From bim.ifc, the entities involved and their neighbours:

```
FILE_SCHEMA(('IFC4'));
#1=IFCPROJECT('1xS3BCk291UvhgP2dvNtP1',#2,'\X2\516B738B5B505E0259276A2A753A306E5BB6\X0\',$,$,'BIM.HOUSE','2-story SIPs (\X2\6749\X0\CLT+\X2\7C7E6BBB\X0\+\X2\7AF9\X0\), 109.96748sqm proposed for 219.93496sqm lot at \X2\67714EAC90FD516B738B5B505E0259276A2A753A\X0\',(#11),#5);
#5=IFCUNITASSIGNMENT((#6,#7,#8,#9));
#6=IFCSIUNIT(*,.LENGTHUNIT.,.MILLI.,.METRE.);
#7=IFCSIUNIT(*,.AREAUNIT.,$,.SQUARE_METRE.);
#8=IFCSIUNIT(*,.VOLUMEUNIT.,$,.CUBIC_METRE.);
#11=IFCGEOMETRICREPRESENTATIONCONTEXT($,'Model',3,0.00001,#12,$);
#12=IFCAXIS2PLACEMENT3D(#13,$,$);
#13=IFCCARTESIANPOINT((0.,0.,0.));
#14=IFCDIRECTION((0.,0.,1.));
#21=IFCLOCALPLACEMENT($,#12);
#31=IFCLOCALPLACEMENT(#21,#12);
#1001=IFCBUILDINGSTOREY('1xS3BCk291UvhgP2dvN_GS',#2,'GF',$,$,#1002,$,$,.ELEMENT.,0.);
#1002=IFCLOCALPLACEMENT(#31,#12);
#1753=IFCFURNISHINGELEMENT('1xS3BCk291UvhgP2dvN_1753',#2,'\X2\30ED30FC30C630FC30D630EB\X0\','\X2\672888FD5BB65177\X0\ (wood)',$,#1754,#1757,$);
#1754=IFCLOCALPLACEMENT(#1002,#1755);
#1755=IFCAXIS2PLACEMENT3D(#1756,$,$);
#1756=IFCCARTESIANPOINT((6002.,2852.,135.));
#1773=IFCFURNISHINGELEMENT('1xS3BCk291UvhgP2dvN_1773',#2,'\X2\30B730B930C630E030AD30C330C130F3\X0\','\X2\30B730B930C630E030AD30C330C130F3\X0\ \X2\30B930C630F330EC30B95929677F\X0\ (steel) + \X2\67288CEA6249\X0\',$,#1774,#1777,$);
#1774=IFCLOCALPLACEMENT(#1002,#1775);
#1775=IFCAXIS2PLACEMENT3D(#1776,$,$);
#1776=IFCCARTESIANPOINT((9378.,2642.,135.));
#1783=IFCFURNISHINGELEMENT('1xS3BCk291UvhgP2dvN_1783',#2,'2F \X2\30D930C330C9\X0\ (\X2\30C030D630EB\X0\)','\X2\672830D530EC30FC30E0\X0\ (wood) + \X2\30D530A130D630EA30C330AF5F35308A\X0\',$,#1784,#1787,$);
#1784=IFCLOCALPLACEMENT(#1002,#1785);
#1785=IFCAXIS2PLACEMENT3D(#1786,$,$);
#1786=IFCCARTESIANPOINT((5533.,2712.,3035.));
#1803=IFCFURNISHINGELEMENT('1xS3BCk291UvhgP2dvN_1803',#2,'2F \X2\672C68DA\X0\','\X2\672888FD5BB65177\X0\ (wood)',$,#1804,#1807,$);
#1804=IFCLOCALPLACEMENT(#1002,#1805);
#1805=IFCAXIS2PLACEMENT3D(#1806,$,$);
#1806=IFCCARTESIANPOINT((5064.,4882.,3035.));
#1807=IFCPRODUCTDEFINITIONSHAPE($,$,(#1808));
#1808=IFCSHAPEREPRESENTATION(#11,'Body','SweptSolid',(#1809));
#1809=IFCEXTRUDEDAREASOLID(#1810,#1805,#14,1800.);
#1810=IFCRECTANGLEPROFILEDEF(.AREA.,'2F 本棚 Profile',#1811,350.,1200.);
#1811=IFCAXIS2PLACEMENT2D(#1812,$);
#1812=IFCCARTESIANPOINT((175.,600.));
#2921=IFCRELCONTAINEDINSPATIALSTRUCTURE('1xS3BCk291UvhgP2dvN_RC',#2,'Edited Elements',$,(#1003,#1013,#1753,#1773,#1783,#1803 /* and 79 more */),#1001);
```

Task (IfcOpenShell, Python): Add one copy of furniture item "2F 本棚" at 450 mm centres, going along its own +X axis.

```python
import ifcopenshell
import ifcopenshell.api.geometry
import ifcopenshell.api.root
import ifcopenshell.util.element
import ifcopenshell.util.placement
import ifcopenshell.util.unit

model = ifcopenshell.open("bim.ifc")
unit_scale = ifcopenshell.util.unit.calculate_unit_scale(model)


def reuse_history(source, copy):
    """copy_class also copies each property set's owner history, people and application; keep the originals."""
    for rel in copy.IsDefinedBy:
        if rel.is_a("IfcRelDefinesByProperties") and (history := rel.RelatingPropertyDefinition.OwnerHistory):
            rel.RelatingPropertyDefinition.OwnerHistory = source.OwnerHistory
            ifcopenshell.util.element.remove_deep2(model, history)


source = model.by_id(1803)
base = ifcopenshell.util.placement.get_local_placement(source.ObjectPlacement)
step = base[:3, 0] * 0.45 / unit_scale

for i in range(1, 2):
    copy = ifcopenshell.api.root.copy_class(model, product=source)
    copy.Representation = ifcopenshell.util.element.copy_deep(
        model, source.Representation, exclude=["IfcGeometricRepresentationContext", "IfcRepresentationMap"]
    )
    reuse_history(source, copy)
    matrix = base.copy()
    matrix[:3, 3] += i * step
    print("added at", matrix[:3, 3].round(3) + 0.0)
    ifcopenshell.api.geometry.edit_object_placement(model, product=copy, matrix=matrix, is_si=False)

model.write("bim_updated.ifc")
```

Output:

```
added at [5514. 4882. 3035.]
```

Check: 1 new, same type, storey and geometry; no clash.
